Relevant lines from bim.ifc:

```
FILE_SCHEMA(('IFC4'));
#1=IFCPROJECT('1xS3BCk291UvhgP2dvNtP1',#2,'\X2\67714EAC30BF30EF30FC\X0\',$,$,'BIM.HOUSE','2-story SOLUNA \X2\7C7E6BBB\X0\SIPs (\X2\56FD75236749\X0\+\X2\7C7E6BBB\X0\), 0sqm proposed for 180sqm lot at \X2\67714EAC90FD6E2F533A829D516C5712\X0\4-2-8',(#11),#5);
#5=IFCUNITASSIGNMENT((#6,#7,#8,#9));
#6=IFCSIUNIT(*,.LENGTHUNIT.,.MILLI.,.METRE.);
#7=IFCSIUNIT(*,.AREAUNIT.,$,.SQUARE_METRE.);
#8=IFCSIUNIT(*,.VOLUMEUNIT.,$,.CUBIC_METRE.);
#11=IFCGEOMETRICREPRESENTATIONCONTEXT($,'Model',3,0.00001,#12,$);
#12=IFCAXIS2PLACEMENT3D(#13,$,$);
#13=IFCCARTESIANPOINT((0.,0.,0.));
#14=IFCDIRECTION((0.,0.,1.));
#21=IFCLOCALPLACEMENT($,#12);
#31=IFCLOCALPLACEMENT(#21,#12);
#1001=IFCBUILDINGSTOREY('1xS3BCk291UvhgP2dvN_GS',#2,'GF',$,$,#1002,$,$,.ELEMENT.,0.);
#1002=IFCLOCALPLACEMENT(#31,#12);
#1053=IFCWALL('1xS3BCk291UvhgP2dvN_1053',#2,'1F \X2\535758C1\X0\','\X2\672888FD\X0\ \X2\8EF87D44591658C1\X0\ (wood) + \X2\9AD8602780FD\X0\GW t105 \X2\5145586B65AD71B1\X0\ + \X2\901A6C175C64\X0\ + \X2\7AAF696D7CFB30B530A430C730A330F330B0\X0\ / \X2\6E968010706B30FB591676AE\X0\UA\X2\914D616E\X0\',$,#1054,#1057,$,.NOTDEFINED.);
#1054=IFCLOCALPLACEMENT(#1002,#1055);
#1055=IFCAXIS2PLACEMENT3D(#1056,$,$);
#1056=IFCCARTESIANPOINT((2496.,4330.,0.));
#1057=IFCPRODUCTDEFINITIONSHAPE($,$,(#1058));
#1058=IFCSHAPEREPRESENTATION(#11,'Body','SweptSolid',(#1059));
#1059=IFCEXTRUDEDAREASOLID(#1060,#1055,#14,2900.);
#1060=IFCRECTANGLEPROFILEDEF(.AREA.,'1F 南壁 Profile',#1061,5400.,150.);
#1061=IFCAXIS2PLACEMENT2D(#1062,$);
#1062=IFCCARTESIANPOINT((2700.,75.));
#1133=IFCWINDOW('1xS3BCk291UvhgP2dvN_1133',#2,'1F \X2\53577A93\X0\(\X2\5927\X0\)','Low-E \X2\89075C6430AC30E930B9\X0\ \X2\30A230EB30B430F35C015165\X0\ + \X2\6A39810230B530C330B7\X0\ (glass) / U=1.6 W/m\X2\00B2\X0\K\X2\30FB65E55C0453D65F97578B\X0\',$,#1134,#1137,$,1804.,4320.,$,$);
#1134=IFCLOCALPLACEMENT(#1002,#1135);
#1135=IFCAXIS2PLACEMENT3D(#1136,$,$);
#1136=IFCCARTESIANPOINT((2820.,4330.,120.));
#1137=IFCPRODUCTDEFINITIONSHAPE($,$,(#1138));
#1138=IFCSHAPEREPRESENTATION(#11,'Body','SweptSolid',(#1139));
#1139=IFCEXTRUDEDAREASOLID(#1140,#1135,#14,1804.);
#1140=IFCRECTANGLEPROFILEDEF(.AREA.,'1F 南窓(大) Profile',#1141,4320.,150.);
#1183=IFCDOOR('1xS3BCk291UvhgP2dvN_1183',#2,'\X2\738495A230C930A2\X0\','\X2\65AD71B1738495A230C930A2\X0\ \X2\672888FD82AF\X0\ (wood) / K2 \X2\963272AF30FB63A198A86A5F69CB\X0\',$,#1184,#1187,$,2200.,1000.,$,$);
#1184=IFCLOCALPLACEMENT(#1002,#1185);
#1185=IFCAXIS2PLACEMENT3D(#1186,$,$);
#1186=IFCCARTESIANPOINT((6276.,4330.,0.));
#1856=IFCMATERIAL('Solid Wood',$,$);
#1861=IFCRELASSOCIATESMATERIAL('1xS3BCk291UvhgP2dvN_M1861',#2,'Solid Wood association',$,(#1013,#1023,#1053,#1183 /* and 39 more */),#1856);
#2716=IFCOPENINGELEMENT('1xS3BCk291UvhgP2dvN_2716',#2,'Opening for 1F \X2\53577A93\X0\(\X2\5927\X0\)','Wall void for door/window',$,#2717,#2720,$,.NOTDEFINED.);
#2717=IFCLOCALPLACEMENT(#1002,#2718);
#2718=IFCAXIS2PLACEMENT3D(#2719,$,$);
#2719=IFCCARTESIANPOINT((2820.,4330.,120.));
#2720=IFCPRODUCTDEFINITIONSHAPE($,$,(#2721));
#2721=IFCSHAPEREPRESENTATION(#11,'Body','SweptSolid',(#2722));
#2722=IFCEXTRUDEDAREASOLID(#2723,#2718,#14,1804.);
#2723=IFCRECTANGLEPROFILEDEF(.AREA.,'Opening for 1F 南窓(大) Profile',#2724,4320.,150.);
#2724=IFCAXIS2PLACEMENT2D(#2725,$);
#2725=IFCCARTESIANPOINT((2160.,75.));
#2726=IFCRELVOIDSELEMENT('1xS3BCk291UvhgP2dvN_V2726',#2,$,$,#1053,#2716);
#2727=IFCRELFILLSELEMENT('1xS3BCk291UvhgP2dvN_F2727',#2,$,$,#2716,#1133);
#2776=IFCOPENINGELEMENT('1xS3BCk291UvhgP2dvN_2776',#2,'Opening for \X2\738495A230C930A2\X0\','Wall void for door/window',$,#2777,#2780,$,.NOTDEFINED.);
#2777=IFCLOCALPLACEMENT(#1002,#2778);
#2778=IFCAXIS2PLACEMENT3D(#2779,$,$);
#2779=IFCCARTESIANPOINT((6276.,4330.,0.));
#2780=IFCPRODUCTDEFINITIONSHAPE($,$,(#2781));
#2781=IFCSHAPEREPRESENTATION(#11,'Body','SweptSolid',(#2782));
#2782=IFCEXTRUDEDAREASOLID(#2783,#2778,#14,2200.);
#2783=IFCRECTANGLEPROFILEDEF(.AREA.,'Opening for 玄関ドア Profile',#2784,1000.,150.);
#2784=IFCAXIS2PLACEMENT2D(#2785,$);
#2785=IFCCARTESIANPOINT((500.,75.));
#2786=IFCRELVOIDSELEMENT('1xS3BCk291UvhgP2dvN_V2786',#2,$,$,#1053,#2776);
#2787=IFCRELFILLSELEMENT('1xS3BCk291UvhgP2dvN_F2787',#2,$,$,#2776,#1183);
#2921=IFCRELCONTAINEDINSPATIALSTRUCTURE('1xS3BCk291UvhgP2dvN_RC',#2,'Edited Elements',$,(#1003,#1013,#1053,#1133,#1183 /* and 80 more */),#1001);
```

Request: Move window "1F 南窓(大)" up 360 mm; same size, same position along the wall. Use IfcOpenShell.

```python
import numpy as np
import ifcopenshell
import ifcopenshell.api.geometry
import ifcopenshell.util.placement
import ifcopenshell.util.unit

model = ifcopenshell.open("bim.ifc")
unit_scale = ifcopenshell.util.unit.calculate_unit_scale(model)

window = model.by_id(1133)
opening = window.FillsVoids[0].RelatingOpeningElement
dz = 360.0

shift = np.array([0.0, 0.0, dz])
# The window is not placed relative to its opening, so move both.
for product in (opening, window):
    matrix = ifcopenshell.util.placement.get_local_placement(product.ObjectPlacement)
    matrix[:3, 3] += shift
    ifcopenshell.api.geometry.edit_object_placement(model, product=product, matrix=matrix, is_si=False)

print(f"moved by {dz * unit_scale:+.3f} m")

model.write("bim-out.ifc")
```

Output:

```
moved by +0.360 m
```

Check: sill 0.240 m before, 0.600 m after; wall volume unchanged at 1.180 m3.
